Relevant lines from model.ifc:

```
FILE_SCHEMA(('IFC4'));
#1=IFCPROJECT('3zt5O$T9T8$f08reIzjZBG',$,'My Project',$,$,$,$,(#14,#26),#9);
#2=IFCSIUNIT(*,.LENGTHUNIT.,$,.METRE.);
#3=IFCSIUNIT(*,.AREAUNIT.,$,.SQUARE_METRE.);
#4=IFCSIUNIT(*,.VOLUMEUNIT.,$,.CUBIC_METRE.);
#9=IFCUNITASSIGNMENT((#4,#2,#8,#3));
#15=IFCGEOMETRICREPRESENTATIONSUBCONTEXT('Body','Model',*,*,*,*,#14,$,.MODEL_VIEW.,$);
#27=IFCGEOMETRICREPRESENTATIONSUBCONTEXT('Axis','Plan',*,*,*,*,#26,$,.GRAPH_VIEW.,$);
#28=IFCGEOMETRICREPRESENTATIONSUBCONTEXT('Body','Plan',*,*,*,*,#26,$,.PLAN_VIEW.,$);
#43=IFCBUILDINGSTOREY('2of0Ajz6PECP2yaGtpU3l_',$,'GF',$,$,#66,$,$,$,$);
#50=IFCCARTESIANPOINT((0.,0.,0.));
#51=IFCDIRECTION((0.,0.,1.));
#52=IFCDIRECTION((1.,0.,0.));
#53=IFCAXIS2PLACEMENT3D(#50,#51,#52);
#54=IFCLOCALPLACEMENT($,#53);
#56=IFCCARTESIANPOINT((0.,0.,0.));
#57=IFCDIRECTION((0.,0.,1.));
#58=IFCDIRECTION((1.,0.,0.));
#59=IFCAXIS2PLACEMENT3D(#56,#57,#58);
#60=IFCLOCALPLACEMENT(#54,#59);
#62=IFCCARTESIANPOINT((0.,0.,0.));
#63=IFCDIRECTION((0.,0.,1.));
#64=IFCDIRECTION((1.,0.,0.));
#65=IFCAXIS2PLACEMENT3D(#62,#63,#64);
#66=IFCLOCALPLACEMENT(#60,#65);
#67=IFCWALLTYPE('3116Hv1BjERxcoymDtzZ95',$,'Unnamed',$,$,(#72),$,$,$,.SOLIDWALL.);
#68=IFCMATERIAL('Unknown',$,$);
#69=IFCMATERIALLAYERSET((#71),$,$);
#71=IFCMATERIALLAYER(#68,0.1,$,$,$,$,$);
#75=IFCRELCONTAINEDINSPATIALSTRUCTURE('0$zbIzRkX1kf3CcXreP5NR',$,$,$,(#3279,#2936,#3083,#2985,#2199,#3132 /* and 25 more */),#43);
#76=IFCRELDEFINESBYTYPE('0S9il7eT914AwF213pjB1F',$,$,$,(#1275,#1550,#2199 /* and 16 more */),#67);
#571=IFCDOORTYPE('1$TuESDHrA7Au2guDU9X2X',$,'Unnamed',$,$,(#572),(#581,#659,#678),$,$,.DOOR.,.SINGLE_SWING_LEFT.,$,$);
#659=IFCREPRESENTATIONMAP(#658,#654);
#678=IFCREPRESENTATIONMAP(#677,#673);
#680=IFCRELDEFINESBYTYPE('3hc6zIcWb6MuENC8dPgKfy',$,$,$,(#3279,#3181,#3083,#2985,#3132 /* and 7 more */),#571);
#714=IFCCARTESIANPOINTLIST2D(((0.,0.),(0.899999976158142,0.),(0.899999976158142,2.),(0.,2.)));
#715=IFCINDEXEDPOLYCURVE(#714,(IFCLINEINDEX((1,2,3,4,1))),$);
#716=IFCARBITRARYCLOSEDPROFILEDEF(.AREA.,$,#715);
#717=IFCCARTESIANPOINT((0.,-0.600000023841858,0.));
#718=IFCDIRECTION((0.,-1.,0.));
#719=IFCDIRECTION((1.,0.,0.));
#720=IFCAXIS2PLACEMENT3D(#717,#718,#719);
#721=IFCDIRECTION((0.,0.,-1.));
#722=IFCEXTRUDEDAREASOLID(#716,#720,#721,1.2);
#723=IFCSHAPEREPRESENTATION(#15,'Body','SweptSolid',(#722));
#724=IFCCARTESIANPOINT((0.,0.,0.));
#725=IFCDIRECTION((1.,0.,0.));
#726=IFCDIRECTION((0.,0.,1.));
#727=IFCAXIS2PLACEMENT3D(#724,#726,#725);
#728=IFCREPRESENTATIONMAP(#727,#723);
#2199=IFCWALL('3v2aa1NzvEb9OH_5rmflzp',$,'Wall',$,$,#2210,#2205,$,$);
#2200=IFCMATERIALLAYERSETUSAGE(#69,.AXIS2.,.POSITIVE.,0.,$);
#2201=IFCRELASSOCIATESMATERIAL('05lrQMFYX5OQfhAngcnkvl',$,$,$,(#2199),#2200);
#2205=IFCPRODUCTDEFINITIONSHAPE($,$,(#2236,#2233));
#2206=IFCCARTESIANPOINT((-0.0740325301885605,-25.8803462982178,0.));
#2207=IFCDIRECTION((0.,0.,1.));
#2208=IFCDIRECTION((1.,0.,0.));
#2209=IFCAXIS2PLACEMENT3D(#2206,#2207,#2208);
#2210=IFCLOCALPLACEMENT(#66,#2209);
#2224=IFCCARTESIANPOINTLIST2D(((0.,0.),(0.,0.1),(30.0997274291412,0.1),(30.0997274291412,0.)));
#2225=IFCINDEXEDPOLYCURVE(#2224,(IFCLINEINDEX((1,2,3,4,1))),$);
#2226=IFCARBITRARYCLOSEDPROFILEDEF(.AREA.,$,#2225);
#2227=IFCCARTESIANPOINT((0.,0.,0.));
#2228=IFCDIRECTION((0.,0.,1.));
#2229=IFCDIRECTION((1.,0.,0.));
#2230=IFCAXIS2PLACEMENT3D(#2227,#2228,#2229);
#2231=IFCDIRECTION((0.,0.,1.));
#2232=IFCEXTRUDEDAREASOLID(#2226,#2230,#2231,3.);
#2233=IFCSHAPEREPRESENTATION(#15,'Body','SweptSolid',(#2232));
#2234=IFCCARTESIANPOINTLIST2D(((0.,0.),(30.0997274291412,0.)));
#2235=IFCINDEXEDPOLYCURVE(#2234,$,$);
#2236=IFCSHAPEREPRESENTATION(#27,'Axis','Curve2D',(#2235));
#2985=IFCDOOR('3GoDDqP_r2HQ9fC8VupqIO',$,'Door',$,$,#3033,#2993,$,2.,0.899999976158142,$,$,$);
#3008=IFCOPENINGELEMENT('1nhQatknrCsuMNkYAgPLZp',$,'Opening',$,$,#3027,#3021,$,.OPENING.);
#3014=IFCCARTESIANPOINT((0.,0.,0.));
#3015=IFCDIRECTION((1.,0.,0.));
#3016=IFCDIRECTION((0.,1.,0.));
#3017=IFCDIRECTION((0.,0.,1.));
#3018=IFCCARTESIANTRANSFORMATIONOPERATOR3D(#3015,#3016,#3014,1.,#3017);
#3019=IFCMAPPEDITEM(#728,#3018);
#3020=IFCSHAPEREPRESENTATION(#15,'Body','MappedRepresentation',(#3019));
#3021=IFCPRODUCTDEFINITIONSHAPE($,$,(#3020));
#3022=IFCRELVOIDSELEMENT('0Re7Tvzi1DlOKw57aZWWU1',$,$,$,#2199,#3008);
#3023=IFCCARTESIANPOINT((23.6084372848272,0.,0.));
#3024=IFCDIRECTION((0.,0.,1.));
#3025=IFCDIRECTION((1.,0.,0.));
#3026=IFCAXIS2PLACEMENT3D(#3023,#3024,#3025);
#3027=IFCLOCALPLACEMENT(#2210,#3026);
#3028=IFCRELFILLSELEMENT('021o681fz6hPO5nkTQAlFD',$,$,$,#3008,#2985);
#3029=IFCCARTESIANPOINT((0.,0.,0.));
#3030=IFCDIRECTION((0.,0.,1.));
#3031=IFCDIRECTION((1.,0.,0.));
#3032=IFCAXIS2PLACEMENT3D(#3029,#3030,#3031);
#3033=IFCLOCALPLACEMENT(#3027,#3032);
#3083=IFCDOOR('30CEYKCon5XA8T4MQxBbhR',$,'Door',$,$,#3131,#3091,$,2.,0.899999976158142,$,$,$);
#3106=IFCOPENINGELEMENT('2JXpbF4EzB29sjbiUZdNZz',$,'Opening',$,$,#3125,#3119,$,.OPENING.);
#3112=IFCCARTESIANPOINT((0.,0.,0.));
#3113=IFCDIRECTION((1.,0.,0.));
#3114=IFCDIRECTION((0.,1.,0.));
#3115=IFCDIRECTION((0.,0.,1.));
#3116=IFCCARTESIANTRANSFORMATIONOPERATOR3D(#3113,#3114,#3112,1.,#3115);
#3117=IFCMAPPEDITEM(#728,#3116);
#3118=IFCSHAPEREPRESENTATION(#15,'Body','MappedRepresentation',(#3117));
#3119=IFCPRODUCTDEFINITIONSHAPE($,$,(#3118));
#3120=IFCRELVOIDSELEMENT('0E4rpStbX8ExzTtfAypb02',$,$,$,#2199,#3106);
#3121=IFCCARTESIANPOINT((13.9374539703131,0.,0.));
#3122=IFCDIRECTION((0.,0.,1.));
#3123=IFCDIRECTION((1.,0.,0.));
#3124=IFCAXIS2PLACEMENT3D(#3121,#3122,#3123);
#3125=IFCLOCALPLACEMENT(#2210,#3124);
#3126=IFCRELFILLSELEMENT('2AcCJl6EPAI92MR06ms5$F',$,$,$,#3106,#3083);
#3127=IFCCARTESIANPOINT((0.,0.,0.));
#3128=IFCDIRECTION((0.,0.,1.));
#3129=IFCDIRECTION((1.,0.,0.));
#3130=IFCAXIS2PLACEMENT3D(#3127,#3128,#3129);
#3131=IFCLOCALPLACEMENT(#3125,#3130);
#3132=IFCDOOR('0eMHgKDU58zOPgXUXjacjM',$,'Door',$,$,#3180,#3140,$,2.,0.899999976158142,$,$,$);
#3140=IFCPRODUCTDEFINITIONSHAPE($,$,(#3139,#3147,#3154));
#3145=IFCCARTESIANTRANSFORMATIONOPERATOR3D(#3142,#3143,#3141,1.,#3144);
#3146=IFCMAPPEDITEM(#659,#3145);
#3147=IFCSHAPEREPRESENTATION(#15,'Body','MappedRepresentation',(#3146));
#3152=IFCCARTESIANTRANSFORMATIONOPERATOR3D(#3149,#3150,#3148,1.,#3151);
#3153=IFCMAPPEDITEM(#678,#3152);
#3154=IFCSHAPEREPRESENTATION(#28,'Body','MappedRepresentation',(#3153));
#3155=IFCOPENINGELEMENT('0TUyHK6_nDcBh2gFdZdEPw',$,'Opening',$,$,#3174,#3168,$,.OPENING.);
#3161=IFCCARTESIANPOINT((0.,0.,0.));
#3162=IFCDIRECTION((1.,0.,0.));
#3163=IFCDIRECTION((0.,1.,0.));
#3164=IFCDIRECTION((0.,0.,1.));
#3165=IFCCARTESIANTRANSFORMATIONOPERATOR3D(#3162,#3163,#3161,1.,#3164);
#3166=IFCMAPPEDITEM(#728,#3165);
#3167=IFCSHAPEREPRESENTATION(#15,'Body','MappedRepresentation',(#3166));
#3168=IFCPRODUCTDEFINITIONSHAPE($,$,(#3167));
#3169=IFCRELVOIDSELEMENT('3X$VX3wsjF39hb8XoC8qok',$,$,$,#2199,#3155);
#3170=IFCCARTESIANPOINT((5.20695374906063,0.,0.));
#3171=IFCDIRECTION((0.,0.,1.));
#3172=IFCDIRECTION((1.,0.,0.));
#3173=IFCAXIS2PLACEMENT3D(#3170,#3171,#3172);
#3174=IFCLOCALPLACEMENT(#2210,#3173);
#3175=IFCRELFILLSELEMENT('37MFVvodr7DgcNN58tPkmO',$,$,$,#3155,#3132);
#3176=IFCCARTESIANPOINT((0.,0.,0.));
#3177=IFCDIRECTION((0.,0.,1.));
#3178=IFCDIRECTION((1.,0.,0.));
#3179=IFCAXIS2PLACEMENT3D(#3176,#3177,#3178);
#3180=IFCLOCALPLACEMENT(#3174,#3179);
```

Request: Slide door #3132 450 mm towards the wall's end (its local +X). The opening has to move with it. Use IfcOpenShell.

```python
import ifcopenshell
import ifcopenshell.api.geometry
import ifcopenshell.util.placement
import ifcopenshell.util.unit

model = ifcopenshell.open("model.ifc")
unit_scale = ifcopenshell.util.unit.calculate_unit_scale(model)

door = model.by_guid("0eMHgKDU58zOPgXUXjacjM")
opening = door.FillsVoids[0].RelatingOpeningElement
wall = opening.VoidsElements[0].RelatingBuildingElement

wall_matrix = ifcopenshell.util.placement.get_local_placement(wall.ObjectPlacement)
shift = wall_matrix[:3, 0] * 0.45 / unit_scale
before = ifcopenshell.util.placement.get_local_placement(door.ObjectPlacement)[:3, 3].copy()

# The door is placed relative to its opening, so it follows when the opening moves.
matrix = ifcopenshell.util.placement.get_local_placement(opening.ObjectPlacement)
matrix[:3, 3] += shift
ifcopenshell.api.geometry.edit_object_placement(
    model, product=opening, matrix=matrix, is_si=False, should_transform_children=True
)

after = ifcopenshell.util.placement.get_local_placement(door.ObjectPlacement)[:3, 3]
print("door moved by", (after - before).round(3) + 0.0)

model.write("model_updated.ifc")
```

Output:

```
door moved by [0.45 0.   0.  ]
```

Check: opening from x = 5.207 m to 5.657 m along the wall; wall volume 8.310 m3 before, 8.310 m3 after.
